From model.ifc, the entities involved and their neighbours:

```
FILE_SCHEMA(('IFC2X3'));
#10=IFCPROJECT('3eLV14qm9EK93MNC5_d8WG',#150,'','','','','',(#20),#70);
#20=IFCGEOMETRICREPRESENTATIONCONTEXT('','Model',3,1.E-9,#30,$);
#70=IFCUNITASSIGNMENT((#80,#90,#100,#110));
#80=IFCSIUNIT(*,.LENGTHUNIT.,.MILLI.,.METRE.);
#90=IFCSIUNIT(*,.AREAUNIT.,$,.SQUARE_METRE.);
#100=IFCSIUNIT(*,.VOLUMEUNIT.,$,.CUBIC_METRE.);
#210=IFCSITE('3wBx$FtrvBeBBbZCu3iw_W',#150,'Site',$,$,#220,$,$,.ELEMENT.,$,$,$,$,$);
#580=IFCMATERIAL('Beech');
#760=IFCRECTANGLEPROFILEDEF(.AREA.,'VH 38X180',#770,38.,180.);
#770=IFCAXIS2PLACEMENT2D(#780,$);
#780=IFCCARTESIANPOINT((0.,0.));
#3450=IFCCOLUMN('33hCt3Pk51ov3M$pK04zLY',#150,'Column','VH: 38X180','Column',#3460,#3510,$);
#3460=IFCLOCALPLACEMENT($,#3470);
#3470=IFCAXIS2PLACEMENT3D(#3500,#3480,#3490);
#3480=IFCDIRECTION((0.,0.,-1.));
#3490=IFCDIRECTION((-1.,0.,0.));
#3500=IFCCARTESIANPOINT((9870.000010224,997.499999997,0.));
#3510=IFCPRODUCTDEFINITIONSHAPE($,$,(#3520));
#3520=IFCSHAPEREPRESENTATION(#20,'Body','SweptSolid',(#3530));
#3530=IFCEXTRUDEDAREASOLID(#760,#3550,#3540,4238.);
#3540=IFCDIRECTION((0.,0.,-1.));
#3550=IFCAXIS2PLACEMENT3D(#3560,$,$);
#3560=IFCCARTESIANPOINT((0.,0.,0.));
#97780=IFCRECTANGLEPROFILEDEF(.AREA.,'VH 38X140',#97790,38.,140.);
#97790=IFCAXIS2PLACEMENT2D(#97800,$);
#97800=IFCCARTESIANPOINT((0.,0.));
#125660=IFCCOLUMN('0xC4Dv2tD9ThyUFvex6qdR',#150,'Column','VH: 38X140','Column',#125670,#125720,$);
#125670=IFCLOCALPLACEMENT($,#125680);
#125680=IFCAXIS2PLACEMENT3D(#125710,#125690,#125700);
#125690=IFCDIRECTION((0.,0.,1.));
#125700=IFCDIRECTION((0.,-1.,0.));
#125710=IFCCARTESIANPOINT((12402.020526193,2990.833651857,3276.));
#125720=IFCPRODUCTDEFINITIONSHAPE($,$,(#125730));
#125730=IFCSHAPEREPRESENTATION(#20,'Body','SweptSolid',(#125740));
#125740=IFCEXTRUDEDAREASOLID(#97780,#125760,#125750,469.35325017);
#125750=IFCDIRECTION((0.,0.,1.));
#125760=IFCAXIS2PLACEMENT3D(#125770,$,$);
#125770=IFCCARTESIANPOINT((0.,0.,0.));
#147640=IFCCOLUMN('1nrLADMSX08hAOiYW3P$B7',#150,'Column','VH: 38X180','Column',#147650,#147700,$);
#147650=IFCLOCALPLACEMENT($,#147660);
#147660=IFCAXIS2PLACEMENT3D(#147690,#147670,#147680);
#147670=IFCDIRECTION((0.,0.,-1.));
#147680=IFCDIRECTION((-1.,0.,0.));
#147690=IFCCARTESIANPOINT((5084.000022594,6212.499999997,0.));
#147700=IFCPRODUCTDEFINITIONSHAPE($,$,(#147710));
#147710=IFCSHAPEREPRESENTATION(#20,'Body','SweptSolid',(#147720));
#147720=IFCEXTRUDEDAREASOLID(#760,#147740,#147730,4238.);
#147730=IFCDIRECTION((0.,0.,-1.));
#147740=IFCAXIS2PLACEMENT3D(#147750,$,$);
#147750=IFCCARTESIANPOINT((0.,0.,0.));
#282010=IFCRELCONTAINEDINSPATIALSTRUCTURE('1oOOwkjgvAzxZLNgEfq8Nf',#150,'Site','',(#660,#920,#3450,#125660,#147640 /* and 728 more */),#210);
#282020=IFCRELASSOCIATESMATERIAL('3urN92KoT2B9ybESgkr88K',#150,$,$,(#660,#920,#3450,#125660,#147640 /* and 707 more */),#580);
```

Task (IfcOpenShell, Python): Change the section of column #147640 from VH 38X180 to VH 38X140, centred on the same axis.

```python
import ifcopenshell
import ifcopenshell.util.element

model = ifcopenshell.open("model.ifc")

member = model.by_guid("1nrLADMSX08hAOiYW3P$B7")
source = next(p for p in model.by_type("IfcRectangleProfileDef") if p.ProfileName == "VH 38X140")

body = next(r for r in member.Representation.Representations if r.RepresentationIdentifier == "Body")
solid = body.Items[0]
old_profile = solid.SweptArea

# Copy the section's sizes but keep this member's own profile position.
profile = ifcopenshell.util.element.copy(model, source)
profile.Position = old_profile.Position
solid.SweptArea = profile
if not model.get_total_inverses(old_profile):
    ifcopenshell.util.element.remove_deep2(model, old_profile)

print(solid.SweptArea)

model.write("model_v2.ifc")
```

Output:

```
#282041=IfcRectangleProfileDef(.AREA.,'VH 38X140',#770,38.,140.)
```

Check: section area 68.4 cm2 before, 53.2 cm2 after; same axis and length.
